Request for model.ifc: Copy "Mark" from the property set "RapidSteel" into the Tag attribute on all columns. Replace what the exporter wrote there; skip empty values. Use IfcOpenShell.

First a look at what the model holds.

```python
import ifcopenshell
import ifcopenshell.util.element

model = ifcopenshell.open("model.ifc")
print(model.schema)
columns = model.by_type("IfcColumn")
print(len(columns), "columns")
for e in columns[:8]:
    source = ifcopenshell.util.element.get_pset(e, "RapidSteel", "Mark")
    target = e.Tag
    print(e.id(), repr(source), repr(target), sep=" | ")
```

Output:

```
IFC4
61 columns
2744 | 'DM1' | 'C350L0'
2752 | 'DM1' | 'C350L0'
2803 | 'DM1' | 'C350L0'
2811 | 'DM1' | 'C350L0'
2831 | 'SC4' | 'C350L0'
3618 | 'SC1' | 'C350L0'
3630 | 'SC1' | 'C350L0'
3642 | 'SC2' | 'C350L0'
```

```python
import ifcopenshell
import ifcopenshell.util.element

model = ifcopenshell.open("model.ifc")

count = 0
for e in model.by_type("IfcColumn"):
    value = ifcopenshell.util.element.get_pset(e, "RapidSteel", "Mark")
    current = e.Tag
    if not value or not value.strip() or current == value:
        continue
    e.Tag = value
    count += 1

print(count, "columns updated")

model.write("model-out.ifc")
```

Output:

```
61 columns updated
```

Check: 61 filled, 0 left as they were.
